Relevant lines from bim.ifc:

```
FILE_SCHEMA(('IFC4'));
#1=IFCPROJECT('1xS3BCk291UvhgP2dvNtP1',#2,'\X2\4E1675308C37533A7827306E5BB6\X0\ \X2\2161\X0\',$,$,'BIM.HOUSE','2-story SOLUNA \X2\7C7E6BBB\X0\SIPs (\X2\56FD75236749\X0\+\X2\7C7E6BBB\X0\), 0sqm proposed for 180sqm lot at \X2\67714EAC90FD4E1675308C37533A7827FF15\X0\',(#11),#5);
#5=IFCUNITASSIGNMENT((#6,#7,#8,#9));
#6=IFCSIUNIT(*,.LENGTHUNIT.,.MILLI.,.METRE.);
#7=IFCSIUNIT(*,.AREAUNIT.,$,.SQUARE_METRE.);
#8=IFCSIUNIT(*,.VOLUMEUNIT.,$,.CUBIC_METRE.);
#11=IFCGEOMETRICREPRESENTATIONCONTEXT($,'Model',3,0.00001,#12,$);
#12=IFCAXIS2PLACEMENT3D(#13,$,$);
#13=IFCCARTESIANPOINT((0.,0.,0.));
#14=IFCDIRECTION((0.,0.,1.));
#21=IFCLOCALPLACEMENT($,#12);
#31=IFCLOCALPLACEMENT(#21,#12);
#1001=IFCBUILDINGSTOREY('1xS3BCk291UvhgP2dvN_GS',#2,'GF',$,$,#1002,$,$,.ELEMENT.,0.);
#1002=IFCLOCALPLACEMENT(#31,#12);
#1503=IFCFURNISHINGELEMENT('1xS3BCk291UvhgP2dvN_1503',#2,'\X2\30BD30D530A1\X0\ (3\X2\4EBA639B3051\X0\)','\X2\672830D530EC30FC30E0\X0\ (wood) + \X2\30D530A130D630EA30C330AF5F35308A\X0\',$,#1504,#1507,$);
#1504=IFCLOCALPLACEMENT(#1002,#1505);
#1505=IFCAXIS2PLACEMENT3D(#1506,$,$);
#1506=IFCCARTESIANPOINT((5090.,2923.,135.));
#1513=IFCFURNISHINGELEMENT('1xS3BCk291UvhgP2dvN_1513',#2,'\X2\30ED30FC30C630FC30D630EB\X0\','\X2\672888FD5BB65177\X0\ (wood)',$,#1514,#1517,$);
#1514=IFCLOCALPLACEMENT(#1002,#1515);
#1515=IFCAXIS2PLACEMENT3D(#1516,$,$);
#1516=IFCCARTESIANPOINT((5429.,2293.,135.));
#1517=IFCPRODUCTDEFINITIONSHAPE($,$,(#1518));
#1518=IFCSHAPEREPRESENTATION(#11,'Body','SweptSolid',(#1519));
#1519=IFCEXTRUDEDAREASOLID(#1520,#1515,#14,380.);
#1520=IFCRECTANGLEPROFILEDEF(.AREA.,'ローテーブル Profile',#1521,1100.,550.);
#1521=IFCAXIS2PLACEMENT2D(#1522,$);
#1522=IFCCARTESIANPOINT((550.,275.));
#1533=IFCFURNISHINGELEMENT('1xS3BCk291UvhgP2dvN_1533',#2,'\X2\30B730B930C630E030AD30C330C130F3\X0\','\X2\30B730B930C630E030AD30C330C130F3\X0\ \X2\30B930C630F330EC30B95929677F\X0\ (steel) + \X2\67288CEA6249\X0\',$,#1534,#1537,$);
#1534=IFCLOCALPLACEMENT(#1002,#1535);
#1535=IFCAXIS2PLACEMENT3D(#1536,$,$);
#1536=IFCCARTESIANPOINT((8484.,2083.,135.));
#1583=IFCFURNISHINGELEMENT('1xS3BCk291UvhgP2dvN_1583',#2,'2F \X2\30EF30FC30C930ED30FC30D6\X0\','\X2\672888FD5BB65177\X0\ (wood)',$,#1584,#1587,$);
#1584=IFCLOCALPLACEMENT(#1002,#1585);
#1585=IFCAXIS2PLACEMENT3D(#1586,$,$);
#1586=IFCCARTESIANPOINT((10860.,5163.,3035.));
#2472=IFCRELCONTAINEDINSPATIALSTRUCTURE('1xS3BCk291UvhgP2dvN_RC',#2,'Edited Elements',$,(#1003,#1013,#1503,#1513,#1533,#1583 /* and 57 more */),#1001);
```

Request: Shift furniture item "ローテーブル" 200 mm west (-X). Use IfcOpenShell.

```python
import ifcopenshell
import ifcopenshell.api.geometry
import ifcopenshell.util.placement
import ifcopenshell.util.unit

model = ifcopenshell.open("bim.ifc")
unit_scale = ifcopenshell.util.unit.calculate_unit_scale(model)

item = model.by_guid("1xS3BCk291UvhgP2dvN_1513")
matrix = ifcopenshell.util.placement.get_local_placement(item.ObjectPlacement)
matrix[0, 3] -= 0.2 / unit_scale
ifcopenshell.api.geometry.edit_object_placement(model, product=item, matrix=matrix, is_si=False)

print(ifcopenshell.util.placement.get_local_placement(item.ObjectPlacement).round(3) + 0.0)

model.write("bim_updated.ifc")
```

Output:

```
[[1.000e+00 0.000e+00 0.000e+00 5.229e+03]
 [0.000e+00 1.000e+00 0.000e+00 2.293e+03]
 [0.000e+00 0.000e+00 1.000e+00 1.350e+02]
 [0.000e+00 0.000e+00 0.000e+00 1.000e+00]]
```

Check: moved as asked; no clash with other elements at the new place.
